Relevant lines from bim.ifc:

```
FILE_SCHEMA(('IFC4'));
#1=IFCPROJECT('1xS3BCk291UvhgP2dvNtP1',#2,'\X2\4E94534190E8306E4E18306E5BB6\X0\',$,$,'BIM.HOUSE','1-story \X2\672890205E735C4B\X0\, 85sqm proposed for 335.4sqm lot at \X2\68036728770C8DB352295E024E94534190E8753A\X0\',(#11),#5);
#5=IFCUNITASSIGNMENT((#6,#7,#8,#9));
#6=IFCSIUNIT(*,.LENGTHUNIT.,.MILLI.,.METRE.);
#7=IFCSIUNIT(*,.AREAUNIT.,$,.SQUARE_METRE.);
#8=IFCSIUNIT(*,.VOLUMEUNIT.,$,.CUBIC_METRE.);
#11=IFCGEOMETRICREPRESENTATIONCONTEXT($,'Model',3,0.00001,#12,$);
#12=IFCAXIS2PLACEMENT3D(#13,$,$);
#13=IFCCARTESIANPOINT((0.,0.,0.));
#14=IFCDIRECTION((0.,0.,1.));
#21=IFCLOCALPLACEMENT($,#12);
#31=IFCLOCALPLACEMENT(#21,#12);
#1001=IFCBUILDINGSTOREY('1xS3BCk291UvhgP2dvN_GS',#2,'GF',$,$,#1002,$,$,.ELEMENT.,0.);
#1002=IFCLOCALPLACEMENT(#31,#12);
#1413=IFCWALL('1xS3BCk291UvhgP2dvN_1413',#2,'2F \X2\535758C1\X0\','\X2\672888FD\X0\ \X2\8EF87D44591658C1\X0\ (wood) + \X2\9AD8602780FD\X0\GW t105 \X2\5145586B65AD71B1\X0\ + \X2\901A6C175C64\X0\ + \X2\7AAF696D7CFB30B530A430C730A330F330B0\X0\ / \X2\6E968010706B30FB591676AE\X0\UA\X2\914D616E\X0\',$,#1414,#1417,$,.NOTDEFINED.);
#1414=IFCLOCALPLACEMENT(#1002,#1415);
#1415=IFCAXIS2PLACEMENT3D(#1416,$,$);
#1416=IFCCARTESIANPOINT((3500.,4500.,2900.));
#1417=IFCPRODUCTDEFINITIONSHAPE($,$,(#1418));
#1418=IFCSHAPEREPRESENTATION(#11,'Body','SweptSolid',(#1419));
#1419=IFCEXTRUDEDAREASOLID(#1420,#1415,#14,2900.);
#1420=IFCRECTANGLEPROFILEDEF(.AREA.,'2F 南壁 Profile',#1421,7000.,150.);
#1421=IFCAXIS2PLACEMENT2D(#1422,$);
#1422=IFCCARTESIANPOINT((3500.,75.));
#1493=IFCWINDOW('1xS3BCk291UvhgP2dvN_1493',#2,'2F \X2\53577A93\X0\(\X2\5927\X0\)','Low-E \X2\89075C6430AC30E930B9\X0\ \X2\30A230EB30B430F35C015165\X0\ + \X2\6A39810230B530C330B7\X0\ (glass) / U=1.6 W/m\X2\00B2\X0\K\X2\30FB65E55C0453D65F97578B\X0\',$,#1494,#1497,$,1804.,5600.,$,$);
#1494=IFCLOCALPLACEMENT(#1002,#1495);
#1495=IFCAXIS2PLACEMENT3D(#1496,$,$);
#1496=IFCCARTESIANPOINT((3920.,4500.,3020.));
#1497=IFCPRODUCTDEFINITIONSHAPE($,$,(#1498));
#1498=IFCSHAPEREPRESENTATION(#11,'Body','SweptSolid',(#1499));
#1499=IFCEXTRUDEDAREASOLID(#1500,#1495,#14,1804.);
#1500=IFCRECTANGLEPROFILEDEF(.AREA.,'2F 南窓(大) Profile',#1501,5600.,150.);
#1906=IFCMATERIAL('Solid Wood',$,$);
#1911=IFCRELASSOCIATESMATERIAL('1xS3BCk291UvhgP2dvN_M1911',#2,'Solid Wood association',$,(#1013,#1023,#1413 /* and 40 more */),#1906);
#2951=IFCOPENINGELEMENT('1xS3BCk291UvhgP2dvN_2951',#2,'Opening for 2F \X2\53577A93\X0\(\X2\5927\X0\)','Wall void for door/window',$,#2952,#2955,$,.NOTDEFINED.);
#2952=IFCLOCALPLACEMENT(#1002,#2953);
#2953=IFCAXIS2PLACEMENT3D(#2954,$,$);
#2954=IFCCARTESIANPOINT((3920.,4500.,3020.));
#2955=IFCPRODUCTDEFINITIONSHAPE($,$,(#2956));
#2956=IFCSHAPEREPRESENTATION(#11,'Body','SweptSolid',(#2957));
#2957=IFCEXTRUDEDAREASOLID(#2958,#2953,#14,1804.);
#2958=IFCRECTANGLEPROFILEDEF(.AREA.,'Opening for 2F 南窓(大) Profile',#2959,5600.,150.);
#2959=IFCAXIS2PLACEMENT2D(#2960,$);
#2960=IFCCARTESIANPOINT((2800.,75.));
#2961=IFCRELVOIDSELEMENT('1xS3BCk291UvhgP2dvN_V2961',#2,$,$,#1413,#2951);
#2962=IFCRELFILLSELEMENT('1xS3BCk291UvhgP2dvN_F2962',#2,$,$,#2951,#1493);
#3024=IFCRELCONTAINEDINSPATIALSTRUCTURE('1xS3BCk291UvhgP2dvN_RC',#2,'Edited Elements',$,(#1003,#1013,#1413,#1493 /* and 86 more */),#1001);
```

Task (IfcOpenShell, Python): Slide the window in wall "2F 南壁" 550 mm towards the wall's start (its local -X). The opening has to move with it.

```python
import ifcopenshell
import ifcopenshell.api.geometry
import ifcopenshell.util.placement

model = ifcopenshell.open("bim.ifc")

window = model.by_guid("1xS3BCk291UvhgP2dvN_1493")
opening = window.FillsVoids[0].RelatingOpeningElement
wall = opening.VoidsElements[0].RelatingBuildingElement

wall_matrix = ifcopenshell.util.placement.get_local_placement(wall.ObjectPlacement)
shift = wall_matrix[:3, 0] * -550.0
before = ifcopenshell.util.placement.get_local_placement(window.ObjectPlacement)[:3, 3].copy()

# The window is not placed relative to its opening, so move both.
for product in (opening, window):
    matrix = ifcopenshell.util.placement.get_local_placement(product.ObjectPlacement)
    matrix[:3, 3] += shift
    ifcopenshell.api.geometry.edit_object_placement(model, product=product, matrix=matrix, is_si=False)

after = ifcopenshell.util.placement.get_local_placement(window.ObjectPlacement)[:3, 3]
print("window moved by", (after - before).round(3) + 0.0)

model.write("bim_updated.ifc")
```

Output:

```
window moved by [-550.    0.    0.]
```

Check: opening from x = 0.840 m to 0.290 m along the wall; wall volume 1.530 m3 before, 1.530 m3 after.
